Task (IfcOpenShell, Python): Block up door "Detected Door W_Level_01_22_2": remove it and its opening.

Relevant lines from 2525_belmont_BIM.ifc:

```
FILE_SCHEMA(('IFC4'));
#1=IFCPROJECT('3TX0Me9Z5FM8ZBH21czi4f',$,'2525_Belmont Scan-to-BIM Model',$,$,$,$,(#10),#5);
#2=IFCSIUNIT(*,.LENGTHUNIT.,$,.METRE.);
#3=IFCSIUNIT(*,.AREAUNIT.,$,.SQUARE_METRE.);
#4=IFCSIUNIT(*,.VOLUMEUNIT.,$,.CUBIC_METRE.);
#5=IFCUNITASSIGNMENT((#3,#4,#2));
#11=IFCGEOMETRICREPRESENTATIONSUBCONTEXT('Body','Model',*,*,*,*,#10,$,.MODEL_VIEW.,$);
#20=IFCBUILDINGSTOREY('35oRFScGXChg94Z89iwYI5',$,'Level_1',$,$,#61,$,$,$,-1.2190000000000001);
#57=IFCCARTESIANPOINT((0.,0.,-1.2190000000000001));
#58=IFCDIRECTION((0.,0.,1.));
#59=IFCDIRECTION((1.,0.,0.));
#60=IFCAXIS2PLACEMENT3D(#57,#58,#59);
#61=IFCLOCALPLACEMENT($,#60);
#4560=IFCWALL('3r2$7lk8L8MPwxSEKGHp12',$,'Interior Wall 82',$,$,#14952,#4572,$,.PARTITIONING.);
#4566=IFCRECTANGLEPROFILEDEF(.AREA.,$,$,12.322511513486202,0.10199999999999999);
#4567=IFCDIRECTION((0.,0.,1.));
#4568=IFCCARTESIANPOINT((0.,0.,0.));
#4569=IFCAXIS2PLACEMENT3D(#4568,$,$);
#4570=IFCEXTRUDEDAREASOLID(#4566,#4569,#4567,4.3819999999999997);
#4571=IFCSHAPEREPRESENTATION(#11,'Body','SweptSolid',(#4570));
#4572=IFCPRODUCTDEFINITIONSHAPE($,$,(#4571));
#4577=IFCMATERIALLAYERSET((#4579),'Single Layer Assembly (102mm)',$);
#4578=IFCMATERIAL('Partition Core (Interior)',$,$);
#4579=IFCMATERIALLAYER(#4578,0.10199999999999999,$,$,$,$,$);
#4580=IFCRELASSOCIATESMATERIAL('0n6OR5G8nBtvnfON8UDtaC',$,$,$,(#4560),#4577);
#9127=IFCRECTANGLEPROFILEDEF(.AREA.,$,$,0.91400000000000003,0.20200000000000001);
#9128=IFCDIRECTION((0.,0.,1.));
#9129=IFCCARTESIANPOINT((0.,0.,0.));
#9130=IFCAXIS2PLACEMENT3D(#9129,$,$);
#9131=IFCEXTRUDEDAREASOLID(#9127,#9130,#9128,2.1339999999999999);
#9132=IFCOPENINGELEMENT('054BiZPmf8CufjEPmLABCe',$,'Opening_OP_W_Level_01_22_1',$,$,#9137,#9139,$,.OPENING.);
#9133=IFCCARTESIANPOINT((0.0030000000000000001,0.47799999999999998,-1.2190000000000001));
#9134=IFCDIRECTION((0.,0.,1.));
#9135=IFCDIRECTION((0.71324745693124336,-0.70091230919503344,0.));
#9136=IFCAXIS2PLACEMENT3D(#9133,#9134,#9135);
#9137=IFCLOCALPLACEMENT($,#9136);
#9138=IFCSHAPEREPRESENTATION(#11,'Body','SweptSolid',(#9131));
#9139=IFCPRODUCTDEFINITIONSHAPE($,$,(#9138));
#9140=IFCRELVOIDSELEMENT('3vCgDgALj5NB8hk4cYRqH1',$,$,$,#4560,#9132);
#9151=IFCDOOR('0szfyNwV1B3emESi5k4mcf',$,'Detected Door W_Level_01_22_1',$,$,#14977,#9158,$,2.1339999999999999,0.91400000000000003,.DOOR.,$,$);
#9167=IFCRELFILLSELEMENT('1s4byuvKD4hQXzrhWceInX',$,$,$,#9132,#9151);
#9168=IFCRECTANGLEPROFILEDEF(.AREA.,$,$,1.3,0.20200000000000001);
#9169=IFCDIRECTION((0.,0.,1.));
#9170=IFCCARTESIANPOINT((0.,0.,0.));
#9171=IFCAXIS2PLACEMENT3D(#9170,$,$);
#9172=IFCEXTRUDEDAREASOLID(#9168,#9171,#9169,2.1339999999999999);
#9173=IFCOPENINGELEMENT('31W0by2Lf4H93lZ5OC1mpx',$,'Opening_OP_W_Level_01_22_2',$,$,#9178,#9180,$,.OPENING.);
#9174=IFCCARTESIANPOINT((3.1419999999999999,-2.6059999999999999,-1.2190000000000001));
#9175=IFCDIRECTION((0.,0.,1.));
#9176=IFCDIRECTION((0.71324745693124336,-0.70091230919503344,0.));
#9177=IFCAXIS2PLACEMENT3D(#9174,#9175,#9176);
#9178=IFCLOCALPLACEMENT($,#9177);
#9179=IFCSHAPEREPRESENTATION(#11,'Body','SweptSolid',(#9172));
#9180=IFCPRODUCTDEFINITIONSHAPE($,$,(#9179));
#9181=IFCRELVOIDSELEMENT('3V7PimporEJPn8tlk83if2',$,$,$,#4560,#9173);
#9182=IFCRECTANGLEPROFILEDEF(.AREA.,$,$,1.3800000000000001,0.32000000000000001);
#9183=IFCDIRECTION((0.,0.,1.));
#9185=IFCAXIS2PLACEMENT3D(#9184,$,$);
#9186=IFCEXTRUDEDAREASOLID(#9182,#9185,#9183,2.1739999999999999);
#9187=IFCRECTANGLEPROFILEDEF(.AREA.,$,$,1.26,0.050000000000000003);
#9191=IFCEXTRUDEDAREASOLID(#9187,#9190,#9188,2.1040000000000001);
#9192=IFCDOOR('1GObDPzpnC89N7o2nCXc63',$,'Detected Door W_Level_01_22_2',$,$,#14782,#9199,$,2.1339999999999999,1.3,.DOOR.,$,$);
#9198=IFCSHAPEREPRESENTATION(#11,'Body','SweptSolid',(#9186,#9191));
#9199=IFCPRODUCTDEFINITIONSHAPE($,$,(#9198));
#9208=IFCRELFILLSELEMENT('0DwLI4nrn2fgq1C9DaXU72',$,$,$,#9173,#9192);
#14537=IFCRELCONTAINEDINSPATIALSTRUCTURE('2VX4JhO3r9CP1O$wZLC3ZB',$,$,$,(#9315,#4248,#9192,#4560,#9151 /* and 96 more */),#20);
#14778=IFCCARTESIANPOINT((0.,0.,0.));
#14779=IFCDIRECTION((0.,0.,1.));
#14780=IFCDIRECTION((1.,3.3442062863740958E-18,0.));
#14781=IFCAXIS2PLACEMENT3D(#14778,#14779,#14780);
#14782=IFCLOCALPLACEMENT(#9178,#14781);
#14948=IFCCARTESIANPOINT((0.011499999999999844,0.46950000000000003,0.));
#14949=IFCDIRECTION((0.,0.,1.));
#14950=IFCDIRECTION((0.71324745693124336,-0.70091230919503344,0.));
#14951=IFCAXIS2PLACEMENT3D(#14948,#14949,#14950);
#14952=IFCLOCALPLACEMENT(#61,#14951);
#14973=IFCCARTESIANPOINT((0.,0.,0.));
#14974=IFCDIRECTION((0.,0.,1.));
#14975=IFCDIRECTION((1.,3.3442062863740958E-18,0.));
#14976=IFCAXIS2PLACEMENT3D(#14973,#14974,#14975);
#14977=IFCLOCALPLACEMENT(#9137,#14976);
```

```python
import ifcopenshell
import ifcopenshell.api.feature
import ifcopenshell.api.root
import ifcopenshell.geom
import ifcopenshell.util.shape

model = ifcopenshell.open("2525_belmont_BIM.ifc")
settings = ifcopenshell.geom.settings()


def volume(element):
    """Net volume in cubic metres, openings subtracted."""
    shape = ifcopenshell.geom.create_shape(settings, element)
    return ifcopenshell.util.shape.get_volume(shape.geometry)


door = model.by_guid("1GObDPzpnC89N7o2nCXc63")
opening = door.FillsVoids[0].RelatingOpeningElement
wall = opening.VoidsElements[0].RelatingBuildingElement
before = volume(wall)

ifcopenshell.api.root.remove_product(model, product=door)
ifcopenshell.api.feature.remove_feature(model, feature=opening)

after = volume(wall)

print(f"wall volume {before:.3f} -> {after:.3f} m3")

model.write("2525_belmont_BIM_edited.ifc")
```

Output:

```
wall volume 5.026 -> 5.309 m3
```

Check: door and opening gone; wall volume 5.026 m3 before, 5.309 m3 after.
